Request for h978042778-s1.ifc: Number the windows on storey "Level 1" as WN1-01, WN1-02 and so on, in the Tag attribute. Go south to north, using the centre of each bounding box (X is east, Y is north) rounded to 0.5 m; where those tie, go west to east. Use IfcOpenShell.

First a look at what the model holds.

```python
import ifcopenshell
import ifcopenshell.util.element
import ifcopenshell.util.placement

model = ifcopenshell.open("h978042778-s1.ifc")
print(model.schema)
storey = next(s for s in model.by_type("IfcBuildingStorey") if s.Name == "Level 1")
windows = [e for e in ifcopenshell.util.element.get_decomposition(storey) if e.is_a("IfcWindow")]
for e in sorted(windows, key=lambda e: e.id()):
    origin = ifcopenshell.util.placement.get_local_placement(e.ObjectPlacement)[:3, 3]
    print(e.id(), e.Tag, e.Name, origin.round(2) + 0.0, sep=" | ")
```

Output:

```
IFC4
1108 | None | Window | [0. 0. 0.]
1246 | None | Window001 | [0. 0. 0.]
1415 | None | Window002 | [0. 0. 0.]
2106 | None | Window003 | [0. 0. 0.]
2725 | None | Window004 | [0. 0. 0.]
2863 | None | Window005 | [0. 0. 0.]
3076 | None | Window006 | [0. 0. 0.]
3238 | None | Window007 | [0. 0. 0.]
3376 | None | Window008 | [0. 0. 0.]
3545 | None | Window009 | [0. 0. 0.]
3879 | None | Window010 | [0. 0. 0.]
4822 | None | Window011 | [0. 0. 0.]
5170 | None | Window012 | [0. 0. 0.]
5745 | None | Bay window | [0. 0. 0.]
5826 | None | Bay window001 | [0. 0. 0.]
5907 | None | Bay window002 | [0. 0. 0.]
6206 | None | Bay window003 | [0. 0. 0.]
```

```python
import ifcopenshell
import ifcopenshell.geom
import ifcopenshell.util.element
import ifcopenshell.util.shape

model = ifcopenshell.open("h978042778-s1.ifc")
settings = ifcopenshell.geom.settings()
settings.set("use-world-coords", True)


def centre(element):
    shape = ifcopenshell.geom.create_shape(settings, element)
    return ifcopenshell.util.shape.get_bbox_centroid(shape.geometry)


storey = next(s for s in model.by_type("IfcBuildingStorey") if s.Name == "Level 1")
windows = [e for e in ifcopenshell.util.element.get_decomposition(storey) if e.is_a("IfcWindow")]

# Insertion points can sit at a corner or the storey origin, so sort by the geometry (in metres).
centres = {e: centre(e) for e in windows}
windows.sort(key=lambda e: (round(centres[e][1] / 0.5), centres[e][0]))

for i, e in enumerate(windows, start=1):
    number = f"WN1-{i:02d}"
    e.Tag = number
    print(e.id(), number)

model.write("h978042778-s1_edited.ifc")
```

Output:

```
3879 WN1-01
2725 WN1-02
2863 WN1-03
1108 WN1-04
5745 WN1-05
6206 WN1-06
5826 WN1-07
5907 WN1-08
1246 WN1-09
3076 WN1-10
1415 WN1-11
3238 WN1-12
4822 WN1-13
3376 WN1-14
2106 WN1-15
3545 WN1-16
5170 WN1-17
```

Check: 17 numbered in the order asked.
